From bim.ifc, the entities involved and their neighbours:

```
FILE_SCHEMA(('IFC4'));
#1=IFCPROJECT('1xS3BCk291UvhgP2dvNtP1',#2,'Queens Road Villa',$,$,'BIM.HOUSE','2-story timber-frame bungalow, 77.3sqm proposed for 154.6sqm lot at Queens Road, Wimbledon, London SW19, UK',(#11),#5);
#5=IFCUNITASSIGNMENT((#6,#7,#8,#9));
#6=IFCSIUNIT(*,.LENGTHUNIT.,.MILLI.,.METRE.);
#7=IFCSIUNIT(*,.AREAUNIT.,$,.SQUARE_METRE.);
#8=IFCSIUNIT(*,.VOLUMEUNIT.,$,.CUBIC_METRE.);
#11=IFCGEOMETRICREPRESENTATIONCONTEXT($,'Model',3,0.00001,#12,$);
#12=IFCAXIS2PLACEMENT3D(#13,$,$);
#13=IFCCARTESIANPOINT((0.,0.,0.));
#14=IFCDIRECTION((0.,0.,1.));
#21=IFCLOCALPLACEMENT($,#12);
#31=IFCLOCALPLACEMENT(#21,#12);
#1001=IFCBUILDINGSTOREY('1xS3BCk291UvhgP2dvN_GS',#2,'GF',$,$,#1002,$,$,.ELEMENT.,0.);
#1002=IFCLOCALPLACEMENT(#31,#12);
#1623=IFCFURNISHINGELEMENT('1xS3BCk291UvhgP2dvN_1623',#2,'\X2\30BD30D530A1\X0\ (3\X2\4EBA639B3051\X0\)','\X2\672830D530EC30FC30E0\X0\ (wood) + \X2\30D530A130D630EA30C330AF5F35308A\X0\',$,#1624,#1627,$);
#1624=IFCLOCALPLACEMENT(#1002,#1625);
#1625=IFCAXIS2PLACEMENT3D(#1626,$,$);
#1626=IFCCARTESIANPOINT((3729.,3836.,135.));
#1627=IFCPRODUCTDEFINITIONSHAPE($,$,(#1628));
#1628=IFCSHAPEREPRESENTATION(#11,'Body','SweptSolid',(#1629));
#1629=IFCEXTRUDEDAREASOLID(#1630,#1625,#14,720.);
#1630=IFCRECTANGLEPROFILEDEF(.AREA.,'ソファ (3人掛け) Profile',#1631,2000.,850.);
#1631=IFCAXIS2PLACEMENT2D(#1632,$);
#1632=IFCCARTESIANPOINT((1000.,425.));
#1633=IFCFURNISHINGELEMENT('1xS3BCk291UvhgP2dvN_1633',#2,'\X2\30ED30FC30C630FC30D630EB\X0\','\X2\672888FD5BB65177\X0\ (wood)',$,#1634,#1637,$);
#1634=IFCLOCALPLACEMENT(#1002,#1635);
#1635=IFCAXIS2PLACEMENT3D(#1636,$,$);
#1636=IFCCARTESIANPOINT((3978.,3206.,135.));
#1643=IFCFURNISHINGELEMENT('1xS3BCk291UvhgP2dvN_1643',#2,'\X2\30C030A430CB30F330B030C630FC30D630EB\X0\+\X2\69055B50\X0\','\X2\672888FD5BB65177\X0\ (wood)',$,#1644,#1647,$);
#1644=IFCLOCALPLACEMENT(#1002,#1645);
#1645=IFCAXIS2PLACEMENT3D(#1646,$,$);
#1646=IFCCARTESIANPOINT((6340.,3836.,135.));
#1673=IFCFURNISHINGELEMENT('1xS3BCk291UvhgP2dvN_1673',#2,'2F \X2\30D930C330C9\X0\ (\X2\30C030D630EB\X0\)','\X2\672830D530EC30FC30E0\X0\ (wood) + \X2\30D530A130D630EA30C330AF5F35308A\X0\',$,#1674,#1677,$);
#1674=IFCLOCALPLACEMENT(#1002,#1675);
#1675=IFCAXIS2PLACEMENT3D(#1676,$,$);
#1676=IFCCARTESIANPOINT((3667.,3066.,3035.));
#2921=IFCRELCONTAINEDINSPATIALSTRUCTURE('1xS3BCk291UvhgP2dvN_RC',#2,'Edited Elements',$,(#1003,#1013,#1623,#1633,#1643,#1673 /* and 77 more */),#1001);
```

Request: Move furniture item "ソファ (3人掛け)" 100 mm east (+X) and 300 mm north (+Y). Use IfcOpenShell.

```python
import ifcopenshell
import ifcopenshell.api.geometry
import ifcopenshell.util.placement
import ifcopenshell.util.unit

model = ifcopenshell.open("bim.ifc")
unit_scale = ifcopenshell.util.unit.calculate_unit_scale(model)

item = model.by_id(1623)
matrix = ifcopenshell.util.placement.get_local_placement(item.ObjectPlacement)
matrix[0, 3] += 0.1 / unit_scale
matrix[1, 3] += 0.3 / unit_scale
ifcopenshell.api.geometry.edit_object_placement(model, product=item, matrix=matrix, is_si=False)

print(ifcopenshell.util.placement.get_local_placement(item.ObjectPlacement).round(3) + 0.0)

model.write("bim_rev.ifc")
```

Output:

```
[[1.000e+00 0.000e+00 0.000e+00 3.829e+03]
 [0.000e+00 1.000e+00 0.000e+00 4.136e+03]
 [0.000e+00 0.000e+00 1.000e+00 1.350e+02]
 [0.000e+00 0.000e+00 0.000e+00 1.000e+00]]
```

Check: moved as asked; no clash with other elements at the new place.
